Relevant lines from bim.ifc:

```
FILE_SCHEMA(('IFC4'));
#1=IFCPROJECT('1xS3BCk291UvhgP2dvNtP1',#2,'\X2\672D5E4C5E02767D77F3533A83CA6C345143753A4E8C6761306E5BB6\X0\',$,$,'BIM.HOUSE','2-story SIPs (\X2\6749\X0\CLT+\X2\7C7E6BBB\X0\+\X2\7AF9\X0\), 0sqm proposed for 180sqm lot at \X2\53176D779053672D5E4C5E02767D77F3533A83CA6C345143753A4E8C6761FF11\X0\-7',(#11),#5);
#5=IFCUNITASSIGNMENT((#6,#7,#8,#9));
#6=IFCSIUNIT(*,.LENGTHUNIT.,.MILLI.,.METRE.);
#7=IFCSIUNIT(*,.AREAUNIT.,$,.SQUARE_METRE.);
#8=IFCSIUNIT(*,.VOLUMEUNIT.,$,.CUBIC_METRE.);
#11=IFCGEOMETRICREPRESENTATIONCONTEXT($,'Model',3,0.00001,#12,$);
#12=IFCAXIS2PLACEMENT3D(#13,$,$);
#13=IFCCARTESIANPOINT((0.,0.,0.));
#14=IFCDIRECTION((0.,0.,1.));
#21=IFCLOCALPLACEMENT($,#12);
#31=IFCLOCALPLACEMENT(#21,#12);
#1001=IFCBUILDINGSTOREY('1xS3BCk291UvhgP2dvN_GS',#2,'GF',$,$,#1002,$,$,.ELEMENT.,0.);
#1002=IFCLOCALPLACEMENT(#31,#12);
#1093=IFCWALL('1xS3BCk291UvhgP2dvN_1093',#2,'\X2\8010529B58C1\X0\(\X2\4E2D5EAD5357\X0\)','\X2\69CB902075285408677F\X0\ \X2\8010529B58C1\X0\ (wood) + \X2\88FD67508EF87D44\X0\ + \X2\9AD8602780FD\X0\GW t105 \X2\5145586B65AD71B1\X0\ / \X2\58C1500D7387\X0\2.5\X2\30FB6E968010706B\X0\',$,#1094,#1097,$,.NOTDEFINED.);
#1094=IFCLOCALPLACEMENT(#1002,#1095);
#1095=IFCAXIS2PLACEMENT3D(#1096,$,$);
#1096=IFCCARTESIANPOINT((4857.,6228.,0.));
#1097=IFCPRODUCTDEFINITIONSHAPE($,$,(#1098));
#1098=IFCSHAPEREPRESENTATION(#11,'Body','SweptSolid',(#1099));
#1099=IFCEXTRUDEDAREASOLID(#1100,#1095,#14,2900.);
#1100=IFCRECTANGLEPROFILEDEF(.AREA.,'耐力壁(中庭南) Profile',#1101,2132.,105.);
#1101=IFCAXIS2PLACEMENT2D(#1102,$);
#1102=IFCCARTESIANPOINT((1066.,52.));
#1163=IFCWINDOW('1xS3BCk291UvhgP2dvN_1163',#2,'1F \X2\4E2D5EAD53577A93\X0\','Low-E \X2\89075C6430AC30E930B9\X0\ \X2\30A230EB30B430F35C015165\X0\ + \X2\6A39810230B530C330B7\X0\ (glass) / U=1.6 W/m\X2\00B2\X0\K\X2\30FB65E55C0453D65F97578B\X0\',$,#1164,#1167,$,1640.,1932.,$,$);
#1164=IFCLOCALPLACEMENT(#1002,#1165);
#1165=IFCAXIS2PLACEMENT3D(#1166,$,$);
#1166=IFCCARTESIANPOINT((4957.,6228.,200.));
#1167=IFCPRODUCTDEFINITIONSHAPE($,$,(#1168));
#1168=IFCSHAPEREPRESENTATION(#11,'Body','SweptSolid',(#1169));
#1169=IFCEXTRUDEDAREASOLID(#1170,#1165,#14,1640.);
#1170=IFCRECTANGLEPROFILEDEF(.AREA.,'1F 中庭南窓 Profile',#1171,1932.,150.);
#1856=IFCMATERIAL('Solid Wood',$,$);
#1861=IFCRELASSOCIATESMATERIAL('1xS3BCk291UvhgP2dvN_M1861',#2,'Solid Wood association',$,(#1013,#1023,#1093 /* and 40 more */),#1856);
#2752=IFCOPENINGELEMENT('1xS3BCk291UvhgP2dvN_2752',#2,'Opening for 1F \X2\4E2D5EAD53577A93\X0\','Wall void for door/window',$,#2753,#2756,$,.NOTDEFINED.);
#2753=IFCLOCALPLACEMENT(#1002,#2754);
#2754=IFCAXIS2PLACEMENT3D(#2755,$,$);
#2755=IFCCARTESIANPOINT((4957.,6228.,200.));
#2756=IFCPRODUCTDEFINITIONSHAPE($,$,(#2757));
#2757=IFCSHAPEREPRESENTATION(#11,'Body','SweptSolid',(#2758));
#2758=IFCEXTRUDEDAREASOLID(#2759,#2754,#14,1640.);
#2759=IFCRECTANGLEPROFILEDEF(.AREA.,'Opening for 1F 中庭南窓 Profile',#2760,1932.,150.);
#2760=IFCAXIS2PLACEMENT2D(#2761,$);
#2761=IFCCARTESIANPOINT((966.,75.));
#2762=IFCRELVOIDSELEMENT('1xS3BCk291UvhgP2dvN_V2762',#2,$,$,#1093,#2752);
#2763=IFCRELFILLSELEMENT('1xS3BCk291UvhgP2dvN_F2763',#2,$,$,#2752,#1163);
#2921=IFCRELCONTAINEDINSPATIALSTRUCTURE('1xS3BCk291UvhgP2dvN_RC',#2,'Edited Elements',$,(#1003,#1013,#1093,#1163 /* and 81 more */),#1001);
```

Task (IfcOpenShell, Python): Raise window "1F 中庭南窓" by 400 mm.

```python
import numpy as np
import ifcopenshell
import ifcopenshell.api.geometry
import ifcopenshell.util.placement
import ifcopenshell.util.unit

model = ifcopenshell.open("bim.ifc")
unit_scale = ifcopenshell.util.unit.calculate_unit_scale(model)

window = model.by_id(1163)
opening = window.FillsVoids[0].RelatingOpeningElement
dz = 0.4 / unit_scale

shift = np.array([0.0, 0.0, dz])
# The window is not placed relative to its opening, so move both.
for product in (opening, window):
    matrix = ifcopenshell.util.placement.get_local_placement(product.ObjectPlacement)
    matrix[:3, 3] += shift
    ifcopenshell.api.geometry.edit_object_placement(model, product=product, matrix=matrix, is_si=False)

print(f"moved by {dz * unit_scale:+.3f} m")

model.write("bim_rev.ifc")
```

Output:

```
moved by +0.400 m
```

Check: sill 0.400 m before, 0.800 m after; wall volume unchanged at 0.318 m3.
